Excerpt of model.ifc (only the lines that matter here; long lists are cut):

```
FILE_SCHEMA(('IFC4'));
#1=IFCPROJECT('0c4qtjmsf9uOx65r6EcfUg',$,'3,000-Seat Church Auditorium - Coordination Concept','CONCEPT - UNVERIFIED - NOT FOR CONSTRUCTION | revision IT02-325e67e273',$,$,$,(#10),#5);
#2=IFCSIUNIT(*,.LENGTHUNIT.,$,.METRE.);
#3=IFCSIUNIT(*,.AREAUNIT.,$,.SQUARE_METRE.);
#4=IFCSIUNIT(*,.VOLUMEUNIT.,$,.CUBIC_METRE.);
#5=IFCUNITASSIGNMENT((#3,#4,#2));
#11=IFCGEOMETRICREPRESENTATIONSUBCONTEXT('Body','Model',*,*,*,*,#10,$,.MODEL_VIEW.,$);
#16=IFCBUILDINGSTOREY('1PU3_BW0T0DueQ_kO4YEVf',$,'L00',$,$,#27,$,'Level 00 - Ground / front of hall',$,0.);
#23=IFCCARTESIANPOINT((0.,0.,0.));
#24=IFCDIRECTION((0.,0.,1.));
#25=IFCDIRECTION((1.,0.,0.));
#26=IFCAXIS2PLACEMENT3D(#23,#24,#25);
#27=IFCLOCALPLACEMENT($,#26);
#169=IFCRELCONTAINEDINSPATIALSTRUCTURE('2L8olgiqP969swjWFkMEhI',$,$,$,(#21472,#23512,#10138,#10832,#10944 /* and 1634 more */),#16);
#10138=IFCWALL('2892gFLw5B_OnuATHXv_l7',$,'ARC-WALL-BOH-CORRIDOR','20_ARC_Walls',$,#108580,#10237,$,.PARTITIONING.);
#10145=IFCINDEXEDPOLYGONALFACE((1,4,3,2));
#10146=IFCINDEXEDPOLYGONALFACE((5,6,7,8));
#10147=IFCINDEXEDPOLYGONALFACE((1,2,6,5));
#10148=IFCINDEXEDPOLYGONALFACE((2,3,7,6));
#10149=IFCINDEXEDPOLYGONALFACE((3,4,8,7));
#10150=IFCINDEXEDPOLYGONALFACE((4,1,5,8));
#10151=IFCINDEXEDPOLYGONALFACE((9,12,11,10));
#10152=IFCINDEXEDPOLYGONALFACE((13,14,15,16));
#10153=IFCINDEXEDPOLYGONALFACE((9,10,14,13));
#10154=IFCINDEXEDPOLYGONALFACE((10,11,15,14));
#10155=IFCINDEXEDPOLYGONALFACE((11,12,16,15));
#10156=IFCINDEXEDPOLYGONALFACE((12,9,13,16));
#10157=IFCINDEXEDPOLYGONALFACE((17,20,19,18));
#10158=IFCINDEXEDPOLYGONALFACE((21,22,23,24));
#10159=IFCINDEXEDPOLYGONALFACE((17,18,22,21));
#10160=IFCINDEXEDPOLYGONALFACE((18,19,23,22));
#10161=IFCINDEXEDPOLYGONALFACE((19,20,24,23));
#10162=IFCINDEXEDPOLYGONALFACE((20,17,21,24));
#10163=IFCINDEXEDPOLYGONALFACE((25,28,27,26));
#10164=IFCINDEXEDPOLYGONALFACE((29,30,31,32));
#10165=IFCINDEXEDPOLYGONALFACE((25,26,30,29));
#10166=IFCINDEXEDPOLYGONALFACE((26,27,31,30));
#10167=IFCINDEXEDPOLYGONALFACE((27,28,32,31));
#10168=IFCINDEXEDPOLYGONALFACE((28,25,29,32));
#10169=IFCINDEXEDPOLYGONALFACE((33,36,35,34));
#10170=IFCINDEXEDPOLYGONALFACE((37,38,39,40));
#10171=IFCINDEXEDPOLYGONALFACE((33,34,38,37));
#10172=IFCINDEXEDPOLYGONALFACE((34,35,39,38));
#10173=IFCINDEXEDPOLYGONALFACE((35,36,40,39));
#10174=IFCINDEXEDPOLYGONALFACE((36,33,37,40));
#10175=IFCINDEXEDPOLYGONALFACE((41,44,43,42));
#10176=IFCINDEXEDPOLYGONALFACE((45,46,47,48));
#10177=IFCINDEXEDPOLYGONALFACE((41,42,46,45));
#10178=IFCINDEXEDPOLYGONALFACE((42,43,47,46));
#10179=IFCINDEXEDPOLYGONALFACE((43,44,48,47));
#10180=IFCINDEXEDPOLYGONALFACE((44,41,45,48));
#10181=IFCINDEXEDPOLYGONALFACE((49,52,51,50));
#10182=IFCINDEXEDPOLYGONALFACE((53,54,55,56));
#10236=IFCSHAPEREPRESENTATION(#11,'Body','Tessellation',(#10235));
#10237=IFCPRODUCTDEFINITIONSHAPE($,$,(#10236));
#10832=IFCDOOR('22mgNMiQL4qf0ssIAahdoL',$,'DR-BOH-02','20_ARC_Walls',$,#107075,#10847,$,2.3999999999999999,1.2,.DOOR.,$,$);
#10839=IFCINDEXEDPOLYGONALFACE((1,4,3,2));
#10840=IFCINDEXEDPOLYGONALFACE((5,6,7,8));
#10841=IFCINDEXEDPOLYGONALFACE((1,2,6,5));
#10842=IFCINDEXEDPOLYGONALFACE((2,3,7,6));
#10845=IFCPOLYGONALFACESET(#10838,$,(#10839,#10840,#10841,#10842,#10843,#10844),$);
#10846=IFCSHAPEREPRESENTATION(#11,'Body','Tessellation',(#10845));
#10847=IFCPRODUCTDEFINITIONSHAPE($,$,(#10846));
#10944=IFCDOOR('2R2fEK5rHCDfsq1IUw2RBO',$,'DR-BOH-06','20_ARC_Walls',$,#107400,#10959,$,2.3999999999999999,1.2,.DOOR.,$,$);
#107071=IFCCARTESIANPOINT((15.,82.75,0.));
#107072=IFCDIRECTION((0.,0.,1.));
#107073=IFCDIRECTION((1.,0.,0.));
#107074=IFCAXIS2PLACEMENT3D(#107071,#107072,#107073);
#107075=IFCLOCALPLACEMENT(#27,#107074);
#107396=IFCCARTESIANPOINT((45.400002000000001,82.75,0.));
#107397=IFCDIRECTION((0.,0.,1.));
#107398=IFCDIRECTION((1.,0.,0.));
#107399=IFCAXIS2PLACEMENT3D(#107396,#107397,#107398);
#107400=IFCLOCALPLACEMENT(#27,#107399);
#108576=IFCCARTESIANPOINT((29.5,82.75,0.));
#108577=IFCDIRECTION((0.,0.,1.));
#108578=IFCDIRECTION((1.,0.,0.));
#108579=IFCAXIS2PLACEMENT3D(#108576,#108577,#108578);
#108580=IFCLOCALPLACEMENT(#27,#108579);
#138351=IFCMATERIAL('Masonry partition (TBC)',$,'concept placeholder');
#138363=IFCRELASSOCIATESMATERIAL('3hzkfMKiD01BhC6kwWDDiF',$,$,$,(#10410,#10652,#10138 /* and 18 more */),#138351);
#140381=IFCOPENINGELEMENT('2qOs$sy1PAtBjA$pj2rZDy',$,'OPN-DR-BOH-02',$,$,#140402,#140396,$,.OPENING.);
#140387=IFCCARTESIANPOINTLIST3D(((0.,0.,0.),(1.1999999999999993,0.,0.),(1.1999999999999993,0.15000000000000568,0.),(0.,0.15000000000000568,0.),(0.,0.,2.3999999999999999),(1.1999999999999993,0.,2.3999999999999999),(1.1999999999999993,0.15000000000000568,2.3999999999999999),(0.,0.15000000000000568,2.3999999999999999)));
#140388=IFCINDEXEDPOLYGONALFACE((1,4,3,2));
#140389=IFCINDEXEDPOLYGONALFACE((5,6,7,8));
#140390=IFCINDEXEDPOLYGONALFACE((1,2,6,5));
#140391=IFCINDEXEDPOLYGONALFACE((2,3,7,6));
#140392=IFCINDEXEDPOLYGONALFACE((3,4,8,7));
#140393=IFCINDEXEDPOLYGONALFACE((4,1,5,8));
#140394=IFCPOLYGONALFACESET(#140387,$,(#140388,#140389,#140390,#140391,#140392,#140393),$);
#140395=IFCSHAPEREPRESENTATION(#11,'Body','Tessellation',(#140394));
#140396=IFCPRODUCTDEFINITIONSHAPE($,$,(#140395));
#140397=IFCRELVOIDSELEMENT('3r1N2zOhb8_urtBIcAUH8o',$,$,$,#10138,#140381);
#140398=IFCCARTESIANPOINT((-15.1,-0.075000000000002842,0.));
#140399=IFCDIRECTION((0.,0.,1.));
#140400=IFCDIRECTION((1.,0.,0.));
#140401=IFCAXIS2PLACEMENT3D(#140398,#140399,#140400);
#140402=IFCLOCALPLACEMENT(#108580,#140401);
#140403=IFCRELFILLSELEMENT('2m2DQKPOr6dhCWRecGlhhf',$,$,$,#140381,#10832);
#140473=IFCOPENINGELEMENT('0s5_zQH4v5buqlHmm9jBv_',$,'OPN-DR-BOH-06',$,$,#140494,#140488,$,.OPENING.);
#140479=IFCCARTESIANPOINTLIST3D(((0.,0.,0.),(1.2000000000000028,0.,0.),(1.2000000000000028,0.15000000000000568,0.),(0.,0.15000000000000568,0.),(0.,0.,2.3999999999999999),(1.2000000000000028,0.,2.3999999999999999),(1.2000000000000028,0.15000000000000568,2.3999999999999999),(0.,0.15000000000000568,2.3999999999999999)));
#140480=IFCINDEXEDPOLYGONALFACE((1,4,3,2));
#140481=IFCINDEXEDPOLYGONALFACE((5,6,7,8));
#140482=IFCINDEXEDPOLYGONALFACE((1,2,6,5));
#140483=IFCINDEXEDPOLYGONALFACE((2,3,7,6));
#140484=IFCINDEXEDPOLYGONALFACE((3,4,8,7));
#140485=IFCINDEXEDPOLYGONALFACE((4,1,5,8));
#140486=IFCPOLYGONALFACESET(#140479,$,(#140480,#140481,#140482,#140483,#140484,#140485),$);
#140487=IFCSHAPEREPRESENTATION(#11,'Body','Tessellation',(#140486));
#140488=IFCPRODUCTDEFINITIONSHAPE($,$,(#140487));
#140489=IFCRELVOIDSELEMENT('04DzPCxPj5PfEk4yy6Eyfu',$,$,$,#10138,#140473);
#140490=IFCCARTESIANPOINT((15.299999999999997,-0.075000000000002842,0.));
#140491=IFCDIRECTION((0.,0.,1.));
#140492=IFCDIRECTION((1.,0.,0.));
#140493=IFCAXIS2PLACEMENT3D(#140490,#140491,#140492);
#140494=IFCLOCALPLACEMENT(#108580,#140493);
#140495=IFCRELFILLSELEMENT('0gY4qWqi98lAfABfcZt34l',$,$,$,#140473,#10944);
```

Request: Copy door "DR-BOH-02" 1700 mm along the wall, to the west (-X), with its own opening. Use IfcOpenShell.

```python
import ifcopenshell
import ifcopenshell.api.feature
import ifcopenshell.api.geometry
import ifcopenshell.api.root
import ifcopenshell.geom
import ifcopenshell.util.element
import ifcopenshell.util.placement
import ifcopenshell.util.shape
import ifcopenshell.util.unit

model = ifcopenshell.open("model.ifc")
unit_scale = ifcopenshell.util.unit.calculate_unit_scale(model)
settings = ifcopenshell.geom.settings()


def volume(element):
    """Net volume in cubic metres, openings subtracted."""
    shape = ifcopenshell.geom.create_shape(settings, element)
    return ifcopenshell.util.shape.get_volume(shape.geometry)


door = model.by_guid("22mgNMiQL4qf0ssIAahdoL")
opening = door.FillsVoids[0].RelatingOpeningElement
wall = opening.VoidsElements[0].RelatingBuildingElement
before = volume(wall)
shift = ifcopenshell.util.placement.get_local_placement(wall.ObjectPlacement)[:3, 0] * -1.7 / unit_scale

# copy_class copies the void relationship, type, container and properties, but no geometry.
new_opening = ifcopenshell.api.root.copy_class(model, product=opening)
new_opening.Representation = ifcopenshell.util.element.copy_deep(
    model, opening.Representation, exclude=["IfcGeometricRepresentationContext", "IfcRepresentationMap"]
)
new_door = ifcopenshell.api.root.copy_class(model, product=door)
new_door.Representation = ifcopenshell.util.element.copy_deep(
    model, door.Representation, exclude=["IfcGeometricRepresentationContext", "IfcRepresentationMap"]
)
ifcopenshell.api.feature.add_filling(model, opening=new_opening, element=new_door)

for old, new in ((opening, new_opening), (door, new_door)):
    matrix = ifcopenshell.util.placement.get_local_placement(old.ObjectPlacement)
    matrix[:3, 3] += shift
    ifcopenshell.api.geometry.edit_object_placement(model, product=new, matrix=matrix, is_si=False)

after = volume(wall)

print(f"wall volume {before:.3f} -> {after:.3f} m3")

model.write("model-out.ifc")
```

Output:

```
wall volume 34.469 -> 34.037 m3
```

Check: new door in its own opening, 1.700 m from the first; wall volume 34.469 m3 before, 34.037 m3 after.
